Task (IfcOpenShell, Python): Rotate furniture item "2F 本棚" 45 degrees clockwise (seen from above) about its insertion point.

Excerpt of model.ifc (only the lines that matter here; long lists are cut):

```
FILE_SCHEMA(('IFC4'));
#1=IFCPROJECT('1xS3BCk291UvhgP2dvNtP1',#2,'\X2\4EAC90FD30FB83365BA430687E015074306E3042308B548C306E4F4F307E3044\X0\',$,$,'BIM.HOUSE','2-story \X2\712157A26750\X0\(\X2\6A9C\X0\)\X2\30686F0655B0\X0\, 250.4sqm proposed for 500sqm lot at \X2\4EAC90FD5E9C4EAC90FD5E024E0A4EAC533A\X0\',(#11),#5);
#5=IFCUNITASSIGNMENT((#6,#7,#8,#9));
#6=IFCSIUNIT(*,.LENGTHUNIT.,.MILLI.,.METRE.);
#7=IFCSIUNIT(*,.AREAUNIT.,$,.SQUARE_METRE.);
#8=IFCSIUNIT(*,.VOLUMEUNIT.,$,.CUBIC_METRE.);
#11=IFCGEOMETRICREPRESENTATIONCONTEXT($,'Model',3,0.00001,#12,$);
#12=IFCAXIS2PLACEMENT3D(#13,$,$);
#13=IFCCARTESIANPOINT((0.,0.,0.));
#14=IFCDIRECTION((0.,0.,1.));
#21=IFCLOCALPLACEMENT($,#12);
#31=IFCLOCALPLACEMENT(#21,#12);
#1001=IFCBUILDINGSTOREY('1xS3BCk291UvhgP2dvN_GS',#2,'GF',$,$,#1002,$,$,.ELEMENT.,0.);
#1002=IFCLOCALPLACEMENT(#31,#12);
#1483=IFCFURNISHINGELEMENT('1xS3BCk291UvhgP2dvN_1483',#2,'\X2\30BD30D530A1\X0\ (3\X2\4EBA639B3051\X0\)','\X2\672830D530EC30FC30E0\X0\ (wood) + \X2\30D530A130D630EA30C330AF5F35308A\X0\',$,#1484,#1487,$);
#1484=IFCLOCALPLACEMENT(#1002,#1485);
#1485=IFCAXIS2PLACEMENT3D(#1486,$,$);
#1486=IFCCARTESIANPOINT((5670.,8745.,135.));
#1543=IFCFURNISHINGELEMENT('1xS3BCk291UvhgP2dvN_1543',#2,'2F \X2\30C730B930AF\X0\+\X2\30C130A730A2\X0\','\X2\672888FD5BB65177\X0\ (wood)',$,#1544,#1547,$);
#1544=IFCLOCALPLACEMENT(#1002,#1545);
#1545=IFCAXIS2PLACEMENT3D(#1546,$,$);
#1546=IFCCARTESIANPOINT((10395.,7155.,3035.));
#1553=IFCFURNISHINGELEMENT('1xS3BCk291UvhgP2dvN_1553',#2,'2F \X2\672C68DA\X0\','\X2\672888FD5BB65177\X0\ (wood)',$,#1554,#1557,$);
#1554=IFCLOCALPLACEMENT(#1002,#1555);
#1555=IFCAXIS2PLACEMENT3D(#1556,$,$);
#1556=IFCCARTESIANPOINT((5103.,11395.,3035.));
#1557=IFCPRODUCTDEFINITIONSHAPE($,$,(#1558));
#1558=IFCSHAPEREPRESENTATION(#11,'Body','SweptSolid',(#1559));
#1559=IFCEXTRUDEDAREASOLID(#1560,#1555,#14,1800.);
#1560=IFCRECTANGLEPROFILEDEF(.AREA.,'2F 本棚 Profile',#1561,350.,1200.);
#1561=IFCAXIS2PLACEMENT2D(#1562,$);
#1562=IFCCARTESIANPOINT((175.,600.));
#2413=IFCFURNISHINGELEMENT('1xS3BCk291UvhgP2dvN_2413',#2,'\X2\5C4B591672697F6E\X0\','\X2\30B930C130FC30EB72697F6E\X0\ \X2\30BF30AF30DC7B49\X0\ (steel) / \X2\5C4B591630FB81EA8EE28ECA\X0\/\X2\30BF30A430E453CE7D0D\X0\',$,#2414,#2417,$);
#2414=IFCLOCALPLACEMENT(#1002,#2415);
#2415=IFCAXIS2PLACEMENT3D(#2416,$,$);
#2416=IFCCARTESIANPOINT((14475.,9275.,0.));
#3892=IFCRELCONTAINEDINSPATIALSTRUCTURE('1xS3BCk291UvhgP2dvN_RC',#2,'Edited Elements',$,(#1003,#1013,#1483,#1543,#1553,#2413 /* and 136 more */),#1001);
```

```python
import ifcopenshell
import ifcopenshell.api.geometry
import ifcopenshell.util.placement

model = ifcopenshell.open("model.ifc")

item = model.by_guid("1xS3BCk291UvhgP2dvN_1553")
matrix = ifcopenshell.util.placement.get_local_placement(item.ObjectPlacement)
matrix = matrix @ ifcopenshell.util.placement.rotation(-45, "Z")
ifcopenshell.api.geometry.edit_object_placement(model, product=item, matrix=matrix, is_si=False)

print(ifcopenshell.util.placement.get_local_placement(item.ObjectPlacement).round(3) + 0.0)

model.write("model-out.ifc")
```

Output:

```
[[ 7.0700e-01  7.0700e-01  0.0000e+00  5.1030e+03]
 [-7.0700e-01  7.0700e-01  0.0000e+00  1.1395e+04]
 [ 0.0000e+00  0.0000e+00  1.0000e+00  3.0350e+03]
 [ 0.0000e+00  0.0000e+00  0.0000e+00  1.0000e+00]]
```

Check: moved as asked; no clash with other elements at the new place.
